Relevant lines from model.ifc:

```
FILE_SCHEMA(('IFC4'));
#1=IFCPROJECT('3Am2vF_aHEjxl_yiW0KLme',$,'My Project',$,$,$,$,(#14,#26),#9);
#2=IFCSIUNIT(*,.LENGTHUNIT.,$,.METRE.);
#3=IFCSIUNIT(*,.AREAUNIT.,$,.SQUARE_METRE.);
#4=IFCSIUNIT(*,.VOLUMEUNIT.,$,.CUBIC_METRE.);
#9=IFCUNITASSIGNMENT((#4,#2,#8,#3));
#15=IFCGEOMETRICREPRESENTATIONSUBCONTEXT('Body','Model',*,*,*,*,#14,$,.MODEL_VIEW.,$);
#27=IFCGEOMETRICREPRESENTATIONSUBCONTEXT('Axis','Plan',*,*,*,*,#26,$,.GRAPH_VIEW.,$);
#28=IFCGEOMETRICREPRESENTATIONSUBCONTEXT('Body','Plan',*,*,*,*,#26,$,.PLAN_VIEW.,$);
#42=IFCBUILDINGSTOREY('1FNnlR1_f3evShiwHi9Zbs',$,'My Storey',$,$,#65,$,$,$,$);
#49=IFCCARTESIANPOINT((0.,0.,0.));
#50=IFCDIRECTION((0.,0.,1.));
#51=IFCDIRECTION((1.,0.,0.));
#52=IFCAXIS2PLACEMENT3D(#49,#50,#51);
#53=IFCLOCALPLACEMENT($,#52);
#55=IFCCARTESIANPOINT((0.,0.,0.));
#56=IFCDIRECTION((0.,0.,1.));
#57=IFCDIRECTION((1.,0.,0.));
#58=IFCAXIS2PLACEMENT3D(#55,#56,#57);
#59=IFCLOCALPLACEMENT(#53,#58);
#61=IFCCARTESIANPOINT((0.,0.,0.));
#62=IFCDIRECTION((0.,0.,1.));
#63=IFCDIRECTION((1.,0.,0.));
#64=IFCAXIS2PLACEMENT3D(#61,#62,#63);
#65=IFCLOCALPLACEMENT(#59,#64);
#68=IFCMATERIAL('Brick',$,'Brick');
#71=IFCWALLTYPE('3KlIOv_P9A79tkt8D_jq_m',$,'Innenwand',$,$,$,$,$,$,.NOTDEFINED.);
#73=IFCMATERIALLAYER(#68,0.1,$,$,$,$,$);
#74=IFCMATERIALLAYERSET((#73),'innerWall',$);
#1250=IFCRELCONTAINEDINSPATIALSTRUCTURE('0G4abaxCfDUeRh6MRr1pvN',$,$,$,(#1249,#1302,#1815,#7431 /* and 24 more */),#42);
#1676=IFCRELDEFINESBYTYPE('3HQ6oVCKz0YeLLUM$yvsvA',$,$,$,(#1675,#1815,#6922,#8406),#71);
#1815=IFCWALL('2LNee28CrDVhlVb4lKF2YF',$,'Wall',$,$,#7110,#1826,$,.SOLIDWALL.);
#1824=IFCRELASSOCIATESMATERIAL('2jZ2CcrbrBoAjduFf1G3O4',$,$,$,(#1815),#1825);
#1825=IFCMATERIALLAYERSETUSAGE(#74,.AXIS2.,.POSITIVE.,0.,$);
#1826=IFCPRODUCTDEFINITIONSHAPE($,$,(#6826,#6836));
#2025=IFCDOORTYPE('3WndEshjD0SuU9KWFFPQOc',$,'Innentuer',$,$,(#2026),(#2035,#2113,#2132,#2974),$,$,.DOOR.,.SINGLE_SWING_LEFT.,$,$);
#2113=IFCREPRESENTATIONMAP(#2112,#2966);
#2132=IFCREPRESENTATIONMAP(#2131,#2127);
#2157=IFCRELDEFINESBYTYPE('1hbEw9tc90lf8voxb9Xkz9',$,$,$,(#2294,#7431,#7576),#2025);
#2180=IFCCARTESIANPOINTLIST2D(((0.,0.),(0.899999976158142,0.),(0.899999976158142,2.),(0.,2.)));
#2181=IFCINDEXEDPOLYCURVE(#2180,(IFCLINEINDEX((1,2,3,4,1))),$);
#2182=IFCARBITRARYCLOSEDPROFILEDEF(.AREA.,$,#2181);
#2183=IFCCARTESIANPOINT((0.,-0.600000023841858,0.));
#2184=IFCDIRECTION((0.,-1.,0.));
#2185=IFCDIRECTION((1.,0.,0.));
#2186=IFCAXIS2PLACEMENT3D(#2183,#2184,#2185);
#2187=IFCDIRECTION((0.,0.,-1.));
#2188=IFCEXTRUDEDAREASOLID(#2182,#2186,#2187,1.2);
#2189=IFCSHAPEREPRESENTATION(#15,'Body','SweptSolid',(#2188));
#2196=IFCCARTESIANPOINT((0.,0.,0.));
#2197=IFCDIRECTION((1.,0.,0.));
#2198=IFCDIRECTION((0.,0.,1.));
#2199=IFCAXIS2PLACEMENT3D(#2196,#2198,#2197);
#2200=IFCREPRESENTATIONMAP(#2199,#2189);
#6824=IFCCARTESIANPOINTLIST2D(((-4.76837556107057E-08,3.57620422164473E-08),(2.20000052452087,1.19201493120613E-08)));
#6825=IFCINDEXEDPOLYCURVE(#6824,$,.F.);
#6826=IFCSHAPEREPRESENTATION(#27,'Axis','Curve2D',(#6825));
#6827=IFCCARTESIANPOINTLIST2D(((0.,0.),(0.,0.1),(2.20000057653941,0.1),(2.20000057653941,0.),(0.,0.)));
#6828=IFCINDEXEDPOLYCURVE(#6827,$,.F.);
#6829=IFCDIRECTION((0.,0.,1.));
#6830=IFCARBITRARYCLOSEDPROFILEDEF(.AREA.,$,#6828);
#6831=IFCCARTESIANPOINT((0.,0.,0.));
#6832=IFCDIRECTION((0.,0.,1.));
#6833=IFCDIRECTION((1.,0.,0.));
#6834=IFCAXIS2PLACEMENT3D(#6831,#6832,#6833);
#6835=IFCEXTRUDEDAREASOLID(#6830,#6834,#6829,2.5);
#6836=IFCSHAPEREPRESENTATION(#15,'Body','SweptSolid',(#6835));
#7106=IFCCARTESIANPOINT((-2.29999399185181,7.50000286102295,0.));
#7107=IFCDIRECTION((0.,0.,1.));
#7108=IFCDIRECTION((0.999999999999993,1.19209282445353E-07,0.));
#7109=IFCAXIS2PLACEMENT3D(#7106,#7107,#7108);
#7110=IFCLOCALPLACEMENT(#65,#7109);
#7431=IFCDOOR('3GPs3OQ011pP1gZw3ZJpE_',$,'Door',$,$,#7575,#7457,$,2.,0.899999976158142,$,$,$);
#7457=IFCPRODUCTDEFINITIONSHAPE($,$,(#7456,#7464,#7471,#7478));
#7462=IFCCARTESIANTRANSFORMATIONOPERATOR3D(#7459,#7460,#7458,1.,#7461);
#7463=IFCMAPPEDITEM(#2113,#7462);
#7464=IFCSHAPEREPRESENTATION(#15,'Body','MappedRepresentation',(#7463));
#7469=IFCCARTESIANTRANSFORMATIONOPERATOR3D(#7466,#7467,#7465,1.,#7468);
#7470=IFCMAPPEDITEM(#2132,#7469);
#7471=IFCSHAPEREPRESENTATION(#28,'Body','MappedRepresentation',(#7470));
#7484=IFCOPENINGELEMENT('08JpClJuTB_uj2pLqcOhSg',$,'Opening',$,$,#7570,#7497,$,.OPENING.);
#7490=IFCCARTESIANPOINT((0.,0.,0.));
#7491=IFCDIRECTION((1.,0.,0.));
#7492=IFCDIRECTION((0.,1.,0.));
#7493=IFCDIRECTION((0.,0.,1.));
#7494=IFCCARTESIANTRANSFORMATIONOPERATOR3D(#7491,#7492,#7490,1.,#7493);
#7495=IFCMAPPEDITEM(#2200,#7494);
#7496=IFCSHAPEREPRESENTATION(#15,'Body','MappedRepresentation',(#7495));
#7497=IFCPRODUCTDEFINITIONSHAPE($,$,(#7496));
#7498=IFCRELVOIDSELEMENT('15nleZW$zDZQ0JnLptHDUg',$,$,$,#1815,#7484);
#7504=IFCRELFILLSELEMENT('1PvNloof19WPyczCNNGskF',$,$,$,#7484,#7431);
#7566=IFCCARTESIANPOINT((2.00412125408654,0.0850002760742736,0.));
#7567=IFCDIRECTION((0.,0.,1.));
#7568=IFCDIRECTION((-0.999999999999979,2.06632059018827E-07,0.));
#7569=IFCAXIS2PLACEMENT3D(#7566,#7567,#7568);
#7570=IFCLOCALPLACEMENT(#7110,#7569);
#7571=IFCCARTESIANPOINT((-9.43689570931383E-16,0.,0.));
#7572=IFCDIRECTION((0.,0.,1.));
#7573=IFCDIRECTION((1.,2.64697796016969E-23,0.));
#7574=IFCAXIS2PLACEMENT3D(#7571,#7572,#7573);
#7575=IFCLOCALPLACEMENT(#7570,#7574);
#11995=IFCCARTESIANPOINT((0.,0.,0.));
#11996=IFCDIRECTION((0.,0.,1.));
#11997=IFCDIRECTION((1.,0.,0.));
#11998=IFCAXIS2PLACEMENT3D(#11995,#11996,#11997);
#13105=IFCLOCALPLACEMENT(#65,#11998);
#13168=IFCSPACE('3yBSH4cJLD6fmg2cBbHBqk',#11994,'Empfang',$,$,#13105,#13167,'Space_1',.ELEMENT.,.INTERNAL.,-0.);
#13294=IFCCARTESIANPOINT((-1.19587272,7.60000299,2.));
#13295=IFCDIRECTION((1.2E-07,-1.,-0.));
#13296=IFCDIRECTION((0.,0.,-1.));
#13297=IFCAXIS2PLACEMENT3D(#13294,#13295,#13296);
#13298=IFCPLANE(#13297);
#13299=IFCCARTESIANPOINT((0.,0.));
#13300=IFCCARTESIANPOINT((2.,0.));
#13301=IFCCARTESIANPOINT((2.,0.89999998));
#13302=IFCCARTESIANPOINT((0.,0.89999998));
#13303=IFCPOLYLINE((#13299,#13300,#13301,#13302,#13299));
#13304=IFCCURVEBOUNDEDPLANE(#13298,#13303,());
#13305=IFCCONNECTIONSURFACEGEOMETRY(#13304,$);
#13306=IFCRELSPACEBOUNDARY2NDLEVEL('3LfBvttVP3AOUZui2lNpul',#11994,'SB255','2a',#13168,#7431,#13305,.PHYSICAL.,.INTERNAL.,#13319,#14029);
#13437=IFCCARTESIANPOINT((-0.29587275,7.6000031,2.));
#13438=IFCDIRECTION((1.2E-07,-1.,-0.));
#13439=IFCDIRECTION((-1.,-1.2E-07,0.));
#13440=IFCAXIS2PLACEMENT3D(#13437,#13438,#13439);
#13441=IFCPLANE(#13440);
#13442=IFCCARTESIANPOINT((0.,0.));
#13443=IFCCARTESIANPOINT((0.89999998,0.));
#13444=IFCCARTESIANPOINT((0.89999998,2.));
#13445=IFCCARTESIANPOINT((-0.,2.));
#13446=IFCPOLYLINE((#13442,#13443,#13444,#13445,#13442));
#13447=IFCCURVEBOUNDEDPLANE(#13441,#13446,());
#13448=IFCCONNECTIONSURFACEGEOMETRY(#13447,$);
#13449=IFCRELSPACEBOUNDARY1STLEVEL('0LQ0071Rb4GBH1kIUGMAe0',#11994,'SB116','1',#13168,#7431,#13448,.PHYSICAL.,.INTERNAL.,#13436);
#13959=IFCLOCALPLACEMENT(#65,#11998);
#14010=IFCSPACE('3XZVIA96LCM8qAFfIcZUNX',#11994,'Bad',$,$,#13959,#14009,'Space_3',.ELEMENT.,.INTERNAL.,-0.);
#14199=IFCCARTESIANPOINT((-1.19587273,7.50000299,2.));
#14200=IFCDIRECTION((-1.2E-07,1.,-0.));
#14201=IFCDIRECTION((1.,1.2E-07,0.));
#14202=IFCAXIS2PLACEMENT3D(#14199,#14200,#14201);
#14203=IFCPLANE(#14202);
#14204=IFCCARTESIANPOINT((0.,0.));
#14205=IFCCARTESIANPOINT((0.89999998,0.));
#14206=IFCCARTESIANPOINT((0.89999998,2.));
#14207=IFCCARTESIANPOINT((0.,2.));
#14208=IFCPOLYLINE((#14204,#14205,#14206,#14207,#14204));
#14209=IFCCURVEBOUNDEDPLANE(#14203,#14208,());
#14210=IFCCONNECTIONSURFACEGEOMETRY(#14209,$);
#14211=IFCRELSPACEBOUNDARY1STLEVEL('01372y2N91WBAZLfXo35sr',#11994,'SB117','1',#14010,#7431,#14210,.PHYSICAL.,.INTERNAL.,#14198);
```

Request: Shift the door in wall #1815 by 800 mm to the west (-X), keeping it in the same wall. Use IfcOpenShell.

```python
import numpy as np
import ifcopenshell
import ifcopenshell.api.geometry
import ifcopenshell.util.placement

model = ifcopenshell.open("model.ifc")

door = model.by_guid("3GPs3OQ011pP1gZw3ZJpE_")
opening = door.FillsVoids[0].RelatingOpeningElement
wall = opening.VoidsElements[0].RelatingBuildingElement

wall_matrix = ifcopenshell.util.placement.get_local_placement(wall.ObjectPlacement)
shift = wall_matrix[:3, 0] * -0.8
before = ifcopenshell.util.placement.get_local_placement(door.ObjectPlacement)[:3, 3].copy()

# The door is placed relative to its opening, so it follows when the opening moves.
matrix = ifcopenshell.util.placement.get_local_placement(opening.ObjectPlacement)
matrix[:3, 3] += shift
ifcopenshell.api.geometry.edit_object_placement(
    model, product=opening, matrix=matrix, is_si=False, should_transform_children=True
)

# Space boundary surfaces are stored in each space's coordinates; move them too.
for rel in door.ProvidesBoundaries:
    if not rel.ConnectionGeometry:
        continue
    surface = rel.ConnectionGeometry.SurfaceOnRelatingElement.BasisSurface
    space_matrix = ifcopenshell.util.placement.get_local_placement(rel.RelatingSpace.ObjectPlacement)
    point = np.array(surface.Position.Location.Coordinates) + space_matrix[:3, :3].T @ shift
    surface.Position = model.createIfcAxis2Placement3D(
        model.createIfcCartesianPoint(point.tolist()), surface.Position.Axis, surface.Position.RefDirection
    )

after = ifcopenshell.util.placement.get_local_placement(door.ObjectPlacement)[:3, 3]
print("door moved by", (after - before).round(3) + 0.0)

model.write("model_updated.ifc")
```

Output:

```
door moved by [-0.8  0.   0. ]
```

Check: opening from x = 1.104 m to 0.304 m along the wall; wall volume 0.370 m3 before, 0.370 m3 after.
